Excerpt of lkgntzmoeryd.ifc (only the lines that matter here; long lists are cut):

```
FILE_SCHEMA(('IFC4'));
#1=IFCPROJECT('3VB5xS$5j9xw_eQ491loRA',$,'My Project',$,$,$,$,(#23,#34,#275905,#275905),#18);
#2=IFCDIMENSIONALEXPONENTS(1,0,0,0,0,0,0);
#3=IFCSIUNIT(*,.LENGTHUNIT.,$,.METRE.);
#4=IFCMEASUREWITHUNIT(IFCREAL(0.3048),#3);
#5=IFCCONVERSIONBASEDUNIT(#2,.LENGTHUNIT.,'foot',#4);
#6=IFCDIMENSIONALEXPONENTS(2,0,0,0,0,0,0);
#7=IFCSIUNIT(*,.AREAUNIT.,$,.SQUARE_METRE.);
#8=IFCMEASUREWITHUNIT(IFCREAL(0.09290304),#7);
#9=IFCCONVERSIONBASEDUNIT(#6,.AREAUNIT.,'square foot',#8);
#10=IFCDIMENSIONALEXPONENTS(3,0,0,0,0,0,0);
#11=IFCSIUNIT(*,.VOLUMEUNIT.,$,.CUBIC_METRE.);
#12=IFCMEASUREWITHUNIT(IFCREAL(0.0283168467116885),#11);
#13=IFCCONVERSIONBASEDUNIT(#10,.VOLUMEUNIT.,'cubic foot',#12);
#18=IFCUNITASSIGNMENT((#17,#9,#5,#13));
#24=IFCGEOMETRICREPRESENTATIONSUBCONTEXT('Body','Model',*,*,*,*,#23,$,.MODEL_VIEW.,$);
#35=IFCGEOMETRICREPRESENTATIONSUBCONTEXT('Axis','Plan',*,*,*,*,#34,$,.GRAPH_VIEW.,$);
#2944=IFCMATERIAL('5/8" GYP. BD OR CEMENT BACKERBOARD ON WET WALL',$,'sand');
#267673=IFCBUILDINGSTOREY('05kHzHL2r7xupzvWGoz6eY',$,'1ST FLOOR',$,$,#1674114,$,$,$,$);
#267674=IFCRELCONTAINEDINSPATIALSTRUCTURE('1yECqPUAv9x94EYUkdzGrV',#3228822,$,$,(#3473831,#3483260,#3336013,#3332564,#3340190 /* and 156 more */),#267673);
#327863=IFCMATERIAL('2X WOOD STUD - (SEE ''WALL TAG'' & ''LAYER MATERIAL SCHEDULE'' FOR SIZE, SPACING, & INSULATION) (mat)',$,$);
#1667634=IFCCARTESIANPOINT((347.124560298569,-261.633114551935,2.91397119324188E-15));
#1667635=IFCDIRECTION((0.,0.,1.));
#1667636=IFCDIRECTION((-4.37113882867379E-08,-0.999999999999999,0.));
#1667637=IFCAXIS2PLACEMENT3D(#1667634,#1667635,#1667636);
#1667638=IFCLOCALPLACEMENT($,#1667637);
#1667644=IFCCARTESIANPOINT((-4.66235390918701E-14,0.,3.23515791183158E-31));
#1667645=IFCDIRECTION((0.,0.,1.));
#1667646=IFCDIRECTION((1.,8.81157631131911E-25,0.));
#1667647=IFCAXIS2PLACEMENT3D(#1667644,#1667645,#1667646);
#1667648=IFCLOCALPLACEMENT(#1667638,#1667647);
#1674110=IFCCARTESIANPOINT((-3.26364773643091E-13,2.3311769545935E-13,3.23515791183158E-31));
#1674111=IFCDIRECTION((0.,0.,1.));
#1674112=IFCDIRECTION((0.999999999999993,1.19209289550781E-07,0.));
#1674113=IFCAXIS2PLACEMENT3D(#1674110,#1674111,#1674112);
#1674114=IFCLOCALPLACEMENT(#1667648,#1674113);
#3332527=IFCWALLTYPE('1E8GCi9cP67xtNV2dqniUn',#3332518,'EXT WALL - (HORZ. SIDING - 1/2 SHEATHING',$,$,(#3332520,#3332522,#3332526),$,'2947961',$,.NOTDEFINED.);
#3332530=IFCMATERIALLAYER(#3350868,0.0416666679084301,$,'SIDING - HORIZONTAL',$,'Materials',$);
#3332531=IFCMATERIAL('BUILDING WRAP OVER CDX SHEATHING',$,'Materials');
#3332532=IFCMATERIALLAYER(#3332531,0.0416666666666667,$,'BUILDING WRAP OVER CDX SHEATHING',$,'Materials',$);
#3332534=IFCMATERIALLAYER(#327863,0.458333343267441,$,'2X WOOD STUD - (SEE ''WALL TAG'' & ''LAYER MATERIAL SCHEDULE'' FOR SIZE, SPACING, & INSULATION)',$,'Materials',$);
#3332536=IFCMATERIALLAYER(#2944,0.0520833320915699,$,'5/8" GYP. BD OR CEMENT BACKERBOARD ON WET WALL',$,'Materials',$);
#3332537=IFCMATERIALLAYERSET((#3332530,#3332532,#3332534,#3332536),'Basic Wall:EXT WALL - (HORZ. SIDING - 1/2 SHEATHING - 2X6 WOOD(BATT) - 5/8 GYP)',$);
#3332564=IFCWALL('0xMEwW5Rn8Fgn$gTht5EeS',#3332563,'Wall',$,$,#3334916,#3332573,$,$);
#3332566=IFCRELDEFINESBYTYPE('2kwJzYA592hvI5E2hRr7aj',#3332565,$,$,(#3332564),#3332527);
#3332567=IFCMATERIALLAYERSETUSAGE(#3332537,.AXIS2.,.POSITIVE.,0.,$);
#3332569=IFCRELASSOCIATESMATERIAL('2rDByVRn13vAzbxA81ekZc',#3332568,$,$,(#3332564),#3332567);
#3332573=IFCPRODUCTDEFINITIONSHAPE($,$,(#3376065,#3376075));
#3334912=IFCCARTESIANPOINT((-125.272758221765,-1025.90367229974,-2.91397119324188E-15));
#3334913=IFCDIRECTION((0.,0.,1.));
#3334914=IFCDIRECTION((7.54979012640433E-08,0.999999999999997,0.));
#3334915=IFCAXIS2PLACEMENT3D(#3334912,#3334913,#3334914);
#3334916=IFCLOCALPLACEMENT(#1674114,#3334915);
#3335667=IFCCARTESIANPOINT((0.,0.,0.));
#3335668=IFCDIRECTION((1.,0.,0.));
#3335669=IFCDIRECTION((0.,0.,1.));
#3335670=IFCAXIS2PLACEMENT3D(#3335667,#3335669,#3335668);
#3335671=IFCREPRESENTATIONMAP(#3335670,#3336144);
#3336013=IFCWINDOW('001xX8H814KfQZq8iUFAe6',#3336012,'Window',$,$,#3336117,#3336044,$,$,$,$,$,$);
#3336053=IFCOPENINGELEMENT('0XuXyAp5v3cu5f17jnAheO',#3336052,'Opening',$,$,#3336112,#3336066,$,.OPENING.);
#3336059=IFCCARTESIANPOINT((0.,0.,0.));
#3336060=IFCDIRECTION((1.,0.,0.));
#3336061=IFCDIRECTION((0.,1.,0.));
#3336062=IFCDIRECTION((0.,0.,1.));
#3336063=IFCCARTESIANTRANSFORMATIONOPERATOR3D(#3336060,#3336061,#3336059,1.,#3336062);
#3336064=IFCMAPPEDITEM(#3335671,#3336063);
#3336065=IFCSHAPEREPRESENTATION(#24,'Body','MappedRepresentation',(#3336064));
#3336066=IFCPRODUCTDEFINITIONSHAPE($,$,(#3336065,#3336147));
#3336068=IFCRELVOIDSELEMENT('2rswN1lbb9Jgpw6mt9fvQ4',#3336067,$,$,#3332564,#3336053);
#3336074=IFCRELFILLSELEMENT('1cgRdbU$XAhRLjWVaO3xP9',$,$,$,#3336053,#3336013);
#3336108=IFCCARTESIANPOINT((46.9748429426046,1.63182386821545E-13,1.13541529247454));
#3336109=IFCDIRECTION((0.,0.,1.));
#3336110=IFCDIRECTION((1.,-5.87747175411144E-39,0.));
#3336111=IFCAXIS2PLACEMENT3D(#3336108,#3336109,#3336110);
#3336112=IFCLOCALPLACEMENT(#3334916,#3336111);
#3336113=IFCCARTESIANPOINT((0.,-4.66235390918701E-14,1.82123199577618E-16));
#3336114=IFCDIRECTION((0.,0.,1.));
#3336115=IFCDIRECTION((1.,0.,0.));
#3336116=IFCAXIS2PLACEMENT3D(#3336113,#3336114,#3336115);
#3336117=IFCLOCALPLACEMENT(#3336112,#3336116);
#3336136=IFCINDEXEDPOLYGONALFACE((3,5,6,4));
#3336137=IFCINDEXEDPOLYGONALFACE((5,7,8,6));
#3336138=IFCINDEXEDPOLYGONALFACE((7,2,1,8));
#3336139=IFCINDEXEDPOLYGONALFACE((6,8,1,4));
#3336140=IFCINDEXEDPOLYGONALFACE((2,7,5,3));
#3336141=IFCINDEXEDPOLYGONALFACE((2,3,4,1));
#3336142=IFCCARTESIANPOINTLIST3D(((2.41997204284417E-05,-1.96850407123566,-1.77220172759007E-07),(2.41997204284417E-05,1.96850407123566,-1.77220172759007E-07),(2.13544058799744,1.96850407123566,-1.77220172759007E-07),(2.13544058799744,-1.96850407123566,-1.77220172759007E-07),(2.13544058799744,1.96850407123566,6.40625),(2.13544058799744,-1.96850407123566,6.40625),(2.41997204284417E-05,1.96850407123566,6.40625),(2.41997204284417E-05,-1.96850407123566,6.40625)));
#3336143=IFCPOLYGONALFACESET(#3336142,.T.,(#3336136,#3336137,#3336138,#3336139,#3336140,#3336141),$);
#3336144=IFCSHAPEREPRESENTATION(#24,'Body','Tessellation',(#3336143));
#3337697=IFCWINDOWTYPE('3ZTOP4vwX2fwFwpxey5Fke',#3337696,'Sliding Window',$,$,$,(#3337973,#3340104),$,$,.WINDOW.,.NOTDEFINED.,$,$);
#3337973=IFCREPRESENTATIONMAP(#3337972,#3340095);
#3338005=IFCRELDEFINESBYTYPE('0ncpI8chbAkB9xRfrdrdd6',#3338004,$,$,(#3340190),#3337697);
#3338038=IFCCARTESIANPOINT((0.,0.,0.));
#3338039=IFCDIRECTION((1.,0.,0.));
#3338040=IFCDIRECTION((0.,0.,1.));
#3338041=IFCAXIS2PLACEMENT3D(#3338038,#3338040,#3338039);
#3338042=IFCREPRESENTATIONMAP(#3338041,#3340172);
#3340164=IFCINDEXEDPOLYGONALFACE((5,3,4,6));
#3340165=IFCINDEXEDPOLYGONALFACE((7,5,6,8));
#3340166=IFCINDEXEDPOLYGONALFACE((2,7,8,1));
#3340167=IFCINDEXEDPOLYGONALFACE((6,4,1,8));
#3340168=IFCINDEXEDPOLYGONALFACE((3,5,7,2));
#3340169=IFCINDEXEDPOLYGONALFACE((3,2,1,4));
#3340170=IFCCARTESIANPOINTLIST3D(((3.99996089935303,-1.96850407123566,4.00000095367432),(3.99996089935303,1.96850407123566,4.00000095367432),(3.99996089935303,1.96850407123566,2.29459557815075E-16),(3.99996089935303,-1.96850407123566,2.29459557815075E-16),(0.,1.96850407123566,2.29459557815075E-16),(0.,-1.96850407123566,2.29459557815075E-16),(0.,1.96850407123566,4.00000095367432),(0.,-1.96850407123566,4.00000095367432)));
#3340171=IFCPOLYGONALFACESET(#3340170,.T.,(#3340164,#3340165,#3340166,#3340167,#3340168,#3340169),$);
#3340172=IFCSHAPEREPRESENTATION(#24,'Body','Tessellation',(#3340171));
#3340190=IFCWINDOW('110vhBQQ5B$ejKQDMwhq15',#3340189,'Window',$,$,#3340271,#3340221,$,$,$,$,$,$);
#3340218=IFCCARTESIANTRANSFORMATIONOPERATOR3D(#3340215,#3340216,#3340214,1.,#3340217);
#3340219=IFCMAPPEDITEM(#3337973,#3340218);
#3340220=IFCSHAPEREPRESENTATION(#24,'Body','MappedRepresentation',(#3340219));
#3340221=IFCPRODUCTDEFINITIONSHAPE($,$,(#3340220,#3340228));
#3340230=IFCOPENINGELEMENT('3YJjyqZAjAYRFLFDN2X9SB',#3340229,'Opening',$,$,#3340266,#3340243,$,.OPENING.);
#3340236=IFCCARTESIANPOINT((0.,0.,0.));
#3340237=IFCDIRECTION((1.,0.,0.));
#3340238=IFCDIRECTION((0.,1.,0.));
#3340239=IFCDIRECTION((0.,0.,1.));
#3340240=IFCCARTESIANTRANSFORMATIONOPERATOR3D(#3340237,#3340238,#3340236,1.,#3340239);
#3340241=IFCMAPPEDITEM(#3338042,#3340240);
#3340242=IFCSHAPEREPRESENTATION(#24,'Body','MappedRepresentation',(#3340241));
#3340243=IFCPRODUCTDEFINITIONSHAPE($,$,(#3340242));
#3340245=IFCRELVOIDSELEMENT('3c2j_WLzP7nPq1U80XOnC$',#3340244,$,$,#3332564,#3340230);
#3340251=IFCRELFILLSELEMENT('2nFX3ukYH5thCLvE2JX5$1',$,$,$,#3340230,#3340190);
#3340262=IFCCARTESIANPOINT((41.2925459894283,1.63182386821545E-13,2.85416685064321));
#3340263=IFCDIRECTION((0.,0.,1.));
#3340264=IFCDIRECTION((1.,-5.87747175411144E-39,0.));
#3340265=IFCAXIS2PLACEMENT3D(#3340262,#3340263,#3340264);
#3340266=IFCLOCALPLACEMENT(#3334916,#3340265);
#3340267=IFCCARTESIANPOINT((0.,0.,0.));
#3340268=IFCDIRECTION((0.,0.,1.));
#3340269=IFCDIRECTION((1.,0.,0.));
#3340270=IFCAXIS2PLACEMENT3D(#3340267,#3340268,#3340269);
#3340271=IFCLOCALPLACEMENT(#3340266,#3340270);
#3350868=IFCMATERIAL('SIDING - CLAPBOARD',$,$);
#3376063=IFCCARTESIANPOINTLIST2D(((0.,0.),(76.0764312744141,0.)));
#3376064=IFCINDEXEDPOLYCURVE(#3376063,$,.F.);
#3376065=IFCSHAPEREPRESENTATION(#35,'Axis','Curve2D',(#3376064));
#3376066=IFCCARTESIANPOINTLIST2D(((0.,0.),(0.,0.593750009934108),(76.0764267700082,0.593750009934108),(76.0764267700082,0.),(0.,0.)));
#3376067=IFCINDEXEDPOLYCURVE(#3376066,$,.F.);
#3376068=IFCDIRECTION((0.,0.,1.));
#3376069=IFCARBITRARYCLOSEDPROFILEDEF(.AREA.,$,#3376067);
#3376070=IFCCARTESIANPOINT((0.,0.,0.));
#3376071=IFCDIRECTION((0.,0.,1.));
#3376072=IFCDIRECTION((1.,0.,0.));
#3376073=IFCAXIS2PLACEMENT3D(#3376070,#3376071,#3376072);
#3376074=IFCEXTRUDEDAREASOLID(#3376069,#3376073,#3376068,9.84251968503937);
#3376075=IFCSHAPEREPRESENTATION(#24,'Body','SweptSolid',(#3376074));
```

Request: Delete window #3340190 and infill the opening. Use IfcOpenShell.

```python
import ifcopenshell
import ifcopenshell.api.feature
import ifcopenshell.api.root
import ifcopenshell.geom
import ifcopenshell.util.shape

model = ifcopenshell.open("lkgntzmoeryd.ifc")
settings = ifcopenshell.geom.settings()


def volume(element):
    """Net volume in cubic metres, openings subtracted."""
    shape = ifcopenshell.geom.create_shape(settings, element)
    return ifcopenshell.util.shape.get_volume(shape.geometry)


window = model.by_guid("110vhBQQ5B$ejKQDMwhq15")
opening = window.FillsVoids[0].RelatingOpeningElement
wall = opening.VoidsElements[0].RelatingBuildingElement
before = volume(wall)

ifcopenshell.api.root.remove_product(model, product=window)
ifcopenshell.api.feature.remove_feature(model, feature=opening)

after = volume(wall)

print(f"wall volume {before:.3f} -> {after:.3f} m3")

model.write("lkgntzmoeryd_rev.ifc")
```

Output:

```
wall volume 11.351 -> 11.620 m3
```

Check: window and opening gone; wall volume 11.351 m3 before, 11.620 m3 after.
